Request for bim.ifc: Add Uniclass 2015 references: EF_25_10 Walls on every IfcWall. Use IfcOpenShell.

First a look at what the model holds.

```python
import ifcopenshell

model = ifcopenshell.open("bim.ifc")
print(model.schema)
print("classifications:", [c.Name for c in model.by_type("IfcClassification")])
for ifc_class in ("IfcDoor", "IfcRoof", "IfcStair", "IfcWall", "IfcWindow"):
    print(ifc_class, len(model.by_type(ifc_class)))
```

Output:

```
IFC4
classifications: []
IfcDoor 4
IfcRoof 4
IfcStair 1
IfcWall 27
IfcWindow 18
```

```python
import ifcopenshell
import ifcopenshell.api.classification

model = ifcopenshell.open("bim.ifc")

system = ifcopenshell.api.classification.add_classification(model, classification="Uniclass 2015")

codes = {
    "IfcWall": ("EF_25_10", "Walls"),
}
for ifc_class, (code, name) in codes.items():
    products = model.by_type(ifc_class)
    ifcopenshell.api.classification.add_reference(
        model, products=products, classification=system, identification=code, name=name
    )
    print(code, len(products))

model.write("bim_v2.ifc")
```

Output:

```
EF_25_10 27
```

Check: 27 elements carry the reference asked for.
